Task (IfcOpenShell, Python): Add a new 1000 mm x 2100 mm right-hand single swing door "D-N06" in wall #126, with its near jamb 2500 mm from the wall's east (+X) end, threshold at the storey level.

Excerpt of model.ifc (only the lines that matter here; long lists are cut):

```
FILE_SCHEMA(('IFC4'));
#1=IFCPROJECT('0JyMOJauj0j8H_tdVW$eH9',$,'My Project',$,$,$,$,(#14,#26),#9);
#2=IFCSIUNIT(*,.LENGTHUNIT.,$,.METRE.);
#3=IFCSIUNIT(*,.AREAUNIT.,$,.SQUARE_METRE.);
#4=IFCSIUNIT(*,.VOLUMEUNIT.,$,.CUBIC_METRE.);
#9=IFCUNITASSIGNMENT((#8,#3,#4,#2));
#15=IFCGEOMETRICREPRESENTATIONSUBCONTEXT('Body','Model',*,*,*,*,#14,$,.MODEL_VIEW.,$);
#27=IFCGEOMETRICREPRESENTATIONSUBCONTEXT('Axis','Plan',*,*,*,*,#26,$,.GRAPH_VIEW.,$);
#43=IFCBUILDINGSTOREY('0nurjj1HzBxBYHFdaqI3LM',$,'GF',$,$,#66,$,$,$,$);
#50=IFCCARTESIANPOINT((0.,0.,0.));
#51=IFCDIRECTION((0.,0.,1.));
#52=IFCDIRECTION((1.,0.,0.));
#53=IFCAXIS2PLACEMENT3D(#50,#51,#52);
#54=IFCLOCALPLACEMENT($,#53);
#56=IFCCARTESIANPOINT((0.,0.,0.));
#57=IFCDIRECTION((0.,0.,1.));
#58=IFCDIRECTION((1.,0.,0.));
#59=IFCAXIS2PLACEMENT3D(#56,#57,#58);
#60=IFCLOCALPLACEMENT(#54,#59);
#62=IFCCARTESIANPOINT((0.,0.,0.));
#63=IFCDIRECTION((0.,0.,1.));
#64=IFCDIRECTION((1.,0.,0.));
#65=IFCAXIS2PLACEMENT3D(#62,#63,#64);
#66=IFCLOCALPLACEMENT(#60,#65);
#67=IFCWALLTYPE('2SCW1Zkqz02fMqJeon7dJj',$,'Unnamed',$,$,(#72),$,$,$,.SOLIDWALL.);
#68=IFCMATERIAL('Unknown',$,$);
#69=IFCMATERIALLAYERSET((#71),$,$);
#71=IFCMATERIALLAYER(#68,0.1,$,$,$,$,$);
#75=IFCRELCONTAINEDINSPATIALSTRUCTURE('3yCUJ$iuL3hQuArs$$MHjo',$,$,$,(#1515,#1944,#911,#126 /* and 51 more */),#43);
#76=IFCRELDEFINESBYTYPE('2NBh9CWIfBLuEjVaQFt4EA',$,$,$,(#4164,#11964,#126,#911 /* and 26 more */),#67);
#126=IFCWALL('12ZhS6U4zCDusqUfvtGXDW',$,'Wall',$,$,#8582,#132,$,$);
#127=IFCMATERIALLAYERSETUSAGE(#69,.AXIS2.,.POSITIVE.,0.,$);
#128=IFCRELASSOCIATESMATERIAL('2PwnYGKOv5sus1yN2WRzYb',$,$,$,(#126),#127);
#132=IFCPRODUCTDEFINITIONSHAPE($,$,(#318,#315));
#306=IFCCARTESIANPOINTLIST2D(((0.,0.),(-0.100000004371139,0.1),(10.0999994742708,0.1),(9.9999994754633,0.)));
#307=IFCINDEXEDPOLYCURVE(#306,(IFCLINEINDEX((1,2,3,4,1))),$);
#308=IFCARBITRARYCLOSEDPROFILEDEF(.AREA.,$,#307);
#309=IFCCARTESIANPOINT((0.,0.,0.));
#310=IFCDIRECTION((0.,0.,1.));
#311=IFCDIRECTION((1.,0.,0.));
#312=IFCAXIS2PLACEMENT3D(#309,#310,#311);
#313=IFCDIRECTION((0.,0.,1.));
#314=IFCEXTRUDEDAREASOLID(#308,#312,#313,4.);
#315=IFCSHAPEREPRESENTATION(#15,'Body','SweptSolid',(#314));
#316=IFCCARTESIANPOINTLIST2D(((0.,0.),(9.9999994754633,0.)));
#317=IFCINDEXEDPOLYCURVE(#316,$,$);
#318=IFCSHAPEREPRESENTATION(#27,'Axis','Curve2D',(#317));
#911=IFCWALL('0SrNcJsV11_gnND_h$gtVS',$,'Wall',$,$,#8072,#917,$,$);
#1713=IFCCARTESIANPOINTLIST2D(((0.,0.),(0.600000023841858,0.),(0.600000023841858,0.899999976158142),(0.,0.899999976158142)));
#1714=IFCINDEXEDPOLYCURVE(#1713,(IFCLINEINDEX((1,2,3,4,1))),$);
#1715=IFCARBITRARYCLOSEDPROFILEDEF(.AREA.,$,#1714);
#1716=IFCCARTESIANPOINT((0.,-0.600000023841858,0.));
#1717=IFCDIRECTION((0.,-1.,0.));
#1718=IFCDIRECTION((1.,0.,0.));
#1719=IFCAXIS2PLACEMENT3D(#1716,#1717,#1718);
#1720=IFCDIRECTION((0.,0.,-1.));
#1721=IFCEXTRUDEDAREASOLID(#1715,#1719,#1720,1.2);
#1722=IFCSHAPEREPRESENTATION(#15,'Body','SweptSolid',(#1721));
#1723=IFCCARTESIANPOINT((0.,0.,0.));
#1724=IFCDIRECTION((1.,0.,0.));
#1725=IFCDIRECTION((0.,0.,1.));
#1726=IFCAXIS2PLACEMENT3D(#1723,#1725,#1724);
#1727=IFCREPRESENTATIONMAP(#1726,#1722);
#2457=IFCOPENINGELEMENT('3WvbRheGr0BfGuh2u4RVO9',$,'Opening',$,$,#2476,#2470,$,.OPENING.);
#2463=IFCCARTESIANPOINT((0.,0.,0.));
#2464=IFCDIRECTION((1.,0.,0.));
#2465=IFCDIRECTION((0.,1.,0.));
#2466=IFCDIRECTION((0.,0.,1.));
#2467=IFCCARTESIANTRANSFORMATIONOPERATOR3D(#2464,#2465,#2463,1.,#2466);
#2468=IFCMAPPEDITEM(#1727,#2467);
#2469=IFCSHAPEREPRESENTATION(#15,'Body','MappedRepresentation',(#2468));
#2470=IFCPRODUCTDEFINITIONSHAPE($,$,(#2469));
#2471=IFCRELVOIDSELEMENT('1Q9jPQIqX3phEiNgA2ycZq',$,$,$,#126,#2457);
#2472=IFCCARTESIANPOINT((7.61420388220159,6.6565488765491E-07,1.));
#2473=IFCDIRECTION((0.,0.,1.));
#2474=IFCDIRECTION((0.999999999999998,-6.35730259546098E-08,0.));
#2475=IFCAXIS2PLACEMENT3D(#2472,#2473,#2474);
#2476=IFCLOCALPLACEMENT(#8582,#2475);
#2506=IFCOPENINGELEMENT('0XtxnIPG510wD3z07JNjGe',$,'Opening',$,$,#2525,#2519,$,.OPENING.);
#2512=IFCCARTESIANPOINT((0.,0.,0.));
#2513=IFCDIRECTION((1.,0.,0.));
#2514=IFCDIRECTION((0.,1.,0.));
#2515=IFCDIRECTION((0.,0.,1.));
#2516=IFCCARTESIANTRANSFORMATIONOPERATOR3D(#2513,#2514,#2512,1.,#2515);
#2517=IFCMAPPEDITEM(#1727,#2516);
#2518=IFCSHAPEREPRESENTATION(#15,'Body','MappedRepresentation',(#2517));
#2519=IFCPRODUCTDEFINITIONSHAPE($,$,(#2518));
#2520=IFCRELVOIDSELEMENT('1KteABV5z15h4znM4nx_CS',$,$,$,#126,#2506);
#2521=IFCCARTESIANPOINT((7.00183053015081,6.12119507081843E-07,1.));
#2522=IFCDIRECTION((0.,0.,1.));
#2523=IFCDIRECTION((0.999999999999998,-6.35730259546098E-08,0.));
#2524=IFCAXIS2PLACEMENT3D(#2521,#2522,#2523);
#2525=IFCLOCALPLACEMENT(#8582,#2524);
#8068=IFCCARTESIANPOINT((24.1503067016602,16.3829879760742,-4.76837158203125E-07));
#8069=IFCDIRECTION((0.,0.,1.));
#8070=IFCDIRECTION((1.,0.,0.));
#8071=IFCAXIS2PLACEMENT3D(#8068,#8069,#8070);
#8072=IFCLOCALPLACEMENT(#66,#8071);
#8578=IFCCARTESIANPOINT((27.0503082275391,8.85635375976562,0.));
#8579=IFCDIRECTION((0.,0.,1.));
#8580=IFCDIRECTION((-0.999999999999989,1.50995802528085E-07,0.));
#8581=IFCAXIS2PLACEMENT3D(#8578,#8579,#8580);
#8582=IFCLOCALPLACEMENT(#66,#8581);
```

```python
import numpy as np
import ifcopenshell
import ifcopenshell.api.feature
import ifcopenshell.api.geometry
import ifcopenshell.api.root
import ifcopenshell.api.spatial
import ifcopenshell.geom
import ifcopenshell.util.element
import ifcopenshell.util.placement
import ifcopenshell.util.representation
import ifcopenshell.util.shape
import ifcopenshell.util.unit

model = ifcopenshell.open("model.ifc")
unit_scale = ifcopenshell.util.unit.calculate_unit_scale(model)
settings = ifcopenshell.geom.settings()


def volume(element):
    """Net volume in cubic metres, openings subtracted."""
    shape = ifcopenshell.geom.create_shape(settings, element)
    return ifcopenshell.util.shape.get_volume(shape.geometry)


wall = model.by_guid("12ZhS6U4zCDusqUfvtGXDW")
storey = ifcopenshell.util.element.get_container(wall, ifc_class="IfcBuildingStorey")
context = ifcopenshell.util.representation.get_context(model, "Model", "Body", "MODEL_VIEW")
before = volume(wall)

width, height, from_end, sill = 1, 2.1, 2.5, 0.0  # metres

# The wall runs along its own X axis, and the end named is its -X end.
wall_shape = ifcopenshell.geom.create_shape(settings, wall)
x, y, z = ifcopenshell.util.shape.get_vertices(wall_shape.geometry).T
start = x.min() + from_end
face, thickness = float(y.min()), float(y.max() - y.min())
wall_matrix = ifcopenshell.util.placement.get_local_placement(wall.ObjectPlacement)
level = ifcopenshell.util.placement.get_local_placement(storey.ObjectPlacement)[2, 3]


def in_wall(x, y):
    """Placement at x, y metres in the wall's axes, at sill height."""
    matrix = wall_matrix.copy()
    matrix[:, 3] = wall_matrix @ np.array([x / unit_scale, y / unit_scale, 0.0, 1.0])
    matrix[2, 3] = level + sill / unit_scale
    return matrix


# Opening: a box that overshoots both wall faces by 50 mm.
opening = ifcopenshell.api.root.create_entity(model, ifc_class="IfcOpeningElement", predefined_type="OPENING")
box = ifcopenshell.api.geometry.add_wall_representation(
    model, context=context, length=width, height=height, thickness=thickness + 0.1
)
ifcopenshell.api.geometry.assign_representation(model, product=opening, representation=box)
ifcopenshell.api.geometry.edit_object_placement(model, product=opening, matrix=in_wall(start, face - 0.05), is_si=False)
ifcopenshell.api.feature.add_feature(model, feature=opening, element=wall)

door = ifcopenshell.api.root.create_entity(model, ifc_class="IfcDoor", name="D-N06", predefined_type="DOOR")
door.OverallWidth, door.OverallHeight = width / unit_scale, height / unit_scale
door.OperationType = "SINGLE_SWING_RIGHT"
body = ifcopenshell.api.geometry.add_door_representation(
    model,
    context=context,
    overall_width=door.OverallWidth,
    overall_height=door.OverallHeight,
    operation_type="SINGLE_SWING_RIGHT",
    lining_properties={"LiningDepth": thickness / unit_scale, "ThresholdDepth": thickness / unit_scale},
)
ifcopenshell.api.geometry.assign_representation(model, product=door, representation=body)
ifcopenshell.api.spatial.assign_container(model, products=[door], relating_structure=storey)
ifcopenshell.api.feature.add_filling(model, opening=opening, element=door)

# The lining spans the wall, so the door starts at the wall face.
ifcopenshell.api.geometry.edit_object_placement(model, product=door, matrix=in_wall(start, face), is_si=False)

after = volume(wall)

print(f"wall volume {before:.3f} -> {after:.3f} m3")

model.write("model_rev.ifc")
```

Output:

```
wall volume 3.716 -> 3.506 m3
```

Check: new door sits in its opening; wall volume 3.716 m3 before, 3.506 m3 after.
